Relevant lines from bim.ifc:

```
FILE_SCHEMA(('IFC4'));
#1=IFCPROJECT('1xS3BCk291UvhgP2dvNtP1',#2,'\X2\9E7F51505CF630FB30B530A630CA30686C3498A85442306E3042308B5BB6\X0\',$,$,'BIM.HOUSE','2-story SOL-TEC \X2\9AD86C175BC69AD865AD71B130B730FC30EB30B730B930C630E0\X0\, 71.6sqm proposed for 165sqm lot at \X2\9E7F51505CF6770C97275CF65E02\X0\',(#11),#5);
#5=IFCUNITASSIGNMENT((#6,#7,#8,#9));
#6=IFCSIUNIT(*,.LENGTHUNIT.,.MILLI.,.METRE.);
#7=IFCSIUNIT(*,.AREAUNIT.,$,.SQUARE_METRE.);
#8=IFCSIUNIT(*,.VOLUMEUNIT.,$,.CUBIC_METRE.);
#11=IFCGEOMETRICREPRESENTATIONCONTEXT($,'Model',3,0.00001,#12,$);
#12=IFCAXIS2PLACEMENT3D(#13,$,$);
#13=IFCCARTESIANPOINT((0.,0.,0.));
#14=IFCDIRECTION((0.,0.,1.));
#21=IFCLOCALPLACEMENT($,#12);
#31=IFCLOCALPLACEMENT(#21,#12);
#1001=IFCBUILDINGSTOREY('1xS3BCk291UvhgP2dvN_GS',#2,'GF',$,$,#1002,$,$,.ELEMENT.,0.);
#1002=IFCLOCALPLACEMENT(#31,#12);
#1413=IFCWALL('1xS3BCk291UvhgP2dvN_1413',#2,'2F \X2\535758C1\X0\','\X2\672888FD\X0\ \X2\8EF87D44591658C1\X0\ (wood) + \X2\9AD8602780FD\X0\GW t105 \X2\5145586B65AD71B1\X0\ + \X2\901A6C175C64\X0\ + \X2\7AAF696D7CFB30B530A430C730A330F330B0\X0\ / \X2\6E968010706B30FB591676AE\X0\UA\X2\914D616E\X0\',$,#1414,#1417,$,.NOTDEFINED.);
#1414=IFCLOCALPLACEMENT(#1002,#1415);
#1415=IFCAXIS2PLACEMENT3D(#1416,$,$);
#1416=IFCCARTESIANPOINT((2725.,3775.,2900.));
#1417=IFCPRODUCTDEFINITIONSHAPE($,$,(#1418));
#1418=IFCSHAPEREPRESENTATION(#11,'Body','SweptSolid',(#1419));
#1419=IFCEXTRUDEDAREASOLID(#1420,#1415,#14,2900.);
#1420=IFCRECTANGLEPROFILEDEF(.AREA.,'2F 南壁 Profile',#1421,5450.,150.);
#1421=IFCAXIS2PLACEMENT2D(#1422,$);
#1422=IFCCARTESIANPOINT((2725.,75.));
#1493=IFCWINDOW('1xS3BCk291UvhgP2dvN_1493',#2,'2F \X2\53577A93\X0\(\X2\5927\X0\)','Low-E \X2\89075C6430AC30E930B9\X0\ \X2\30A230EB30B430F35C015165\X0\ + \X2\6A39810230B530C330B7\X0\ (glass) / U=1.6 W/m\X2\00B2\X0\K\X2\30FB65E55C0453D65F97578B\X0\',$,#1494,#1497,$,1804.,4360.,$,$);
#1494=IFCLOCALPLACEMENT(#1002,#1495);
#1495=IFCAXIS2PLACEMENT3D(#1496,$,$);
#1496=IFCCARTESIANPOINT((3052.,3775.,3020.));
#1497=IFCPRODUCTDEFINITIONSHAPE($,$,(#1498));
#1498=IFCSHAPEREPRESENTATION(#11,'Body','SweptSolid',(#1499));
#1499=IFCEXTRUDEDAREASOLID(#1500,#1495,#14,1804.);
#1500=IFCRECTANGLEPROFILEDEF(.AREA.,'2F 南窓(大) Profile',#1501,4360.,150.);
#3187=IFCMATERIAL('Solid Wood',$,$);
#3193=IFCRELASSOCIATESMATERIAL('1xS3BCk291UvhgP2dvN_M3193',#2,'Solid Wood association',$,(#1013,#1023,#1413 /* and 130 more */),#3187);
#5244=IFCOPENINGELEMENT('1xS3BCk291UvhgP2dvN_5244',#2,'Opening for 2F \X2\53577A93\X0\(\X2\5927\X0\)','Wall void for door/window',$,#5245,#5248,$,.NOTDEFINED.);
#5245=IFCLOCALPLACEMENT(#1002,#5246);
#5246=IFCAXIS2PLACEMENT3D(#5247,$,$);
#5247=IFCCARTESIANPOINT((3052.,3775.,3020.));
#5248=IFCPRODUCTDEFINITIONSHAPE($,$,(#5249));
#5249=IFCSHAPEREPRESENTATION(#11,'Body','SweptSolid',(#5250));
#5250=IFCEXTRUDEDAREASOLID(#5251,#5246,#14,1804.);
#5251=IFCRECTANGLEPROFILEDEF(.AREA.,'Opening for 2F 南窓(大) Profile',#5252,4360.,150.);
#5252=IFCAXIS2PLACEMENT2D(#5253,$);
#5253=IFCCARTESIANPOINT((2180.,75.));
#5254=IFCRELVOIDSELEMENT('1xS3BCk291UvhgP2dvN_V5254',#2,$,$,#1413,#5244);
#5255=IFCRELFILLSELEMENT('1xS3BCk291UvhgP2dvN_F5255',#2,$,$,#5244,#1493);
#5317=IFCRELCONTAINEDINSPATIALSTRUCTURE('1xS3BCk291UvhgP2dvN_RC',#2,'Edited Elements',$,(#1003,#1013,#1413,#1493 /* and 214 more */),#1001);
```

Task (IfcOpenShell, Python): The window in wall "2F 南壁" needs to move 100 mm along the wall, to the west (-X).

```python
import ifcopenshell
import ifcopenshell.api.geometry
import ifcopenshell.util.placement
import ifcopenshell.util.unit

model = ifcopenshell.open("bim.ifc")
unit_scale = ifcopenshell.util.unit.calculate_unit_scale(model)

window = model.by_guid("1xS3BCk291UvhgP2dvN_1493")
opening = window.FillsVoids[0].RelatingOpeningElement
wall = opening.VoidsElements[0].RelatingBuildingElement

wall_matrix = ifcopenshell.util.placement.get_local_placement(wall.ObjectPlacement)
shift = wall_matrix[:3, 0] * -0.1 / unit_scale
before = ifcopenshell.util.placement.get_local_placement(window.ObjectPlacement)[:3, 3].copy()

# The window is not placed relative to its opening, so move both.
for product in (opening, window):
    matrix = ifcopenshell.util.placement.get_local_placement(product.ObjectPlacement)
    matrix[:3, 3] += shift
    ifcopenshell.api.geometry.edit_object_placement(model, product=product, matrix=matrix, is_si=False)

after = ifcopenshell.util.placement.get_local_placement(window.ObjectPlacement)[:3, 3]
print("window moved by", (after - before).round(3) + 0.0)

model.write("bim-out.ifc")
```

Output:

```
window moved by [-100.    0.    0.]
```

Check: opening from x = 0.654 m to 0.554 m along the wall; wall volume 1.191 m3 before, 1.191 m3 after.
